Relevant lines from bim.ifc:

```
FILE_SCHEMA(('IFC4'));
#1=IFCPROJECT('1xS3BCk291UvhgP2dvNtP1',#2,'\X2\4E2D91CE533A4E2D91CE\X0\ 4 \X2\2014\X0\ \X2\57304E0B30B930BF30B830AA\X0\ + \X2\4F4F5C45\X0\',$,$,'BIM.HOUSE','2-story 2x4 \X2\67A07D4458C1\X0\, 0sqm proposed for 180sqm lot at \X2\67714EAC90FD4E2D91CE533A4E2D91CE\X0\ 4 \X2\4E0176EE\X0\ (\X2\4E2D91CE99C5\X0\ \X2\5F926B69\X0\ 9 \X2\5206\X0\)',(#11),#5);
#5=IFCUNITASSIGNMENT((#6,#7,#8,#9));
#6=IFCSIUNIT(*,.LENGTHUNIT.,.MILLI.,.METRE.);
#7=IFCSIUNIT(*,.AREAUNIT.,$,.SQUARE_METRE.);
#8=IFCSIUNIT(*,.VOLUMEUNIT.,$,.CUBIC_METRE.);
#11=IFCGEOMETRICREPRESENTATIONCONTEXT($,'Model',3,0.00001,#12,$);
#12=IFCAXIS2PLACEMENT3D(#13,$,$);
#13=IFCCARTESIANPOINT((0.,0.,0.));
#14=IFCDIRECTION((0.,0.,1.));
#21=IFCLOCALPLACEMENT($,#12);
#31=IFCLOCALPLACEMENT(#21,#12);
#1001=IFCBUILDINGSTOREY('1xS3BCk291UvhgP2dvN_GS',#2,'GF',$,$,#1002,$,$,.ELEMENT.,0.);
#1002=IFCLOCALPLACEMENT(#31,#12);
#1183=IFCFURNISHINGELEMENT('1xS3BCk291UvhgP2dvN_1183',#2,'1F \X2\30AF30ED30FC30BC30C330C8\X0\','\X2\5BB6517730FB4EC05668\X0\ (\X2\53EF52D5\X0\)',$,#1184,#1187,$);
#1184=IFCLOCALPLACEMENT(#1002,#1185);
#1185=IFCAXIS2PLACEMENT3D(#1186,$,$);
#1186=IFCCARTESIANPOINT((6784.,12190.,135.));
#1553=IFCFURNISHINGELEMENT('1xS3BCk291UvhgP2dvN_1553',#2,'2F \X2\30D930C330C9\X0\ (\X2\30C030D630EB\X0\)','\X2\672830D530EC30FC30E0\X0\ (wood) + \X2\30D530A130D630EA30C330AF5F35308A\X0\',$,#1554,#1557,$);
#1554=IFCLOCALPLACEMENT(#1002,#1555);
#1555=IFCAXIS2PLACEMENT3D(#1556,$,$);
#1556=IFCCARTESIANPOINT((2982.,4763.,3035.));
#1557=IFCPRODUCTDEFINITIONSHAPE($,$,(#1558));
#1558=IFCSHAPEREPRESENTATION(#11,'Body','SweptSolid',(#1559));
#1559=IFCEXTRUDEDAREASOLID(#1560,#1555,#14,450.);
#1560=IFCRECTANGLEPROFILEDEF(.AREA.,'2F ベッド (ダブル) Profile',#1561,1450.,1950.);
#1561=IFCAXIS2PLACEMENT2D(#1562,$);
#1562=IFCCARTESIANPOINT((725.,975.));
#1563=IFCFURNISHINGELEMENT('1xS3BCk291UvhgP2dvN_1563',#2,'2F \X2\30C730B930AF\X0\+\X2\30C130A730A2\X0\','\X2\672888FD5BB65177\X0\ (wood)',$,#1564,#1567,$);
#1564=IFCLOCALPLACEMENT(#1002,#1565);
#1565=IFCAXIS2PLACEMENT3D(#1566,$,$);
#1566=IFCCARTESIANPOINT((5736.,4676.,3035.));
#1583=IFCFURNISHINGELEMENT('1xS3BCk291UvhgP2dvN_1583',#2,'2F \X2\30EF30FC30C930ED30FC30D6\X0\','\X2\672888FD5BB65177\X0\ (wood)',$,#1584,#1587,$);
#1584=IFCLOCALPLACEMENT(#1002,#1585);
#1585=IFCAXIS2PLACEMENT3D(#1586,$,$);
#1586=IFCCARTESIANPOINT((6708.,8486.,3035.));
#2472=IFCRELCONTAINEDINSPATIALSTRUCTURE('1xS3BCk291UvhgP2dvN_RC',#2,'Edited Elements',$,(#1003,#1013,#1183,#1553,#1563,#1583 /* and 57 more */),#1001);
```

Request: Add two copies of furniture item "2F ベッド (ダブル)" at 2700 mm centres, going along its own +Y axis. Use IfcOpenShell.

```python
import ifcopenshell
import ifcopenshell.api.geometry
import ifcopenshell.api.root
import ifcopenshell.util.element
import ifcopenshell.util.placement

model = ifcopenshell.open("bim.ifc")


def reuse_history(source, copy):
    """copy_class also copies each property set's owner history, people and application; keep the originals."""
    for rel in copy.IsDefinedBy:
        if rel.is_a("IfcRelDefinesByProperties") and (history := rel.RelatingPropertyDefinition.OwnerHistory):
            rel.RelatingPropertyDefinition.OwnerHistory = source.OwnerHistory
            ifcopenshell.util.element.remove_deep2(model, history)


source = model.by_guid("1xS3BCk291UvhgP2dvN_1553")
base = ifcopenshell.util.placement.get_local_placement(source.ObjectPlacement)
step = base[:3, 1] * 2700.0

for i in range(1, 3):
    copy = ifcopenshell.api.root.copy_class(model, product=source)
    copy.Representation = ifcopenshell.util.element.copy_deep(
        model, source.Representation, exclude=["IfcGeometricRepresentationContext", "IfcRepresentationMap"]
    )
    reuse_history(source, copy)
    matrix = base.copy()
    matrix[:3, 3] += i * step
    print("added at", matrix[:3, 3].round(3) + 0.0)
    ifcopenshell.api.geometry.edit_object_placement(model, product=copy, matrix=matrix, is_si=False)

model.write("bim_edited.ifc")
```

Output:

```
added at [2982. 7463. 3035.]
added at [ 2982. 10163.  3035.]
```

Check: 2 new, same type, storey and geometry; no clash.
